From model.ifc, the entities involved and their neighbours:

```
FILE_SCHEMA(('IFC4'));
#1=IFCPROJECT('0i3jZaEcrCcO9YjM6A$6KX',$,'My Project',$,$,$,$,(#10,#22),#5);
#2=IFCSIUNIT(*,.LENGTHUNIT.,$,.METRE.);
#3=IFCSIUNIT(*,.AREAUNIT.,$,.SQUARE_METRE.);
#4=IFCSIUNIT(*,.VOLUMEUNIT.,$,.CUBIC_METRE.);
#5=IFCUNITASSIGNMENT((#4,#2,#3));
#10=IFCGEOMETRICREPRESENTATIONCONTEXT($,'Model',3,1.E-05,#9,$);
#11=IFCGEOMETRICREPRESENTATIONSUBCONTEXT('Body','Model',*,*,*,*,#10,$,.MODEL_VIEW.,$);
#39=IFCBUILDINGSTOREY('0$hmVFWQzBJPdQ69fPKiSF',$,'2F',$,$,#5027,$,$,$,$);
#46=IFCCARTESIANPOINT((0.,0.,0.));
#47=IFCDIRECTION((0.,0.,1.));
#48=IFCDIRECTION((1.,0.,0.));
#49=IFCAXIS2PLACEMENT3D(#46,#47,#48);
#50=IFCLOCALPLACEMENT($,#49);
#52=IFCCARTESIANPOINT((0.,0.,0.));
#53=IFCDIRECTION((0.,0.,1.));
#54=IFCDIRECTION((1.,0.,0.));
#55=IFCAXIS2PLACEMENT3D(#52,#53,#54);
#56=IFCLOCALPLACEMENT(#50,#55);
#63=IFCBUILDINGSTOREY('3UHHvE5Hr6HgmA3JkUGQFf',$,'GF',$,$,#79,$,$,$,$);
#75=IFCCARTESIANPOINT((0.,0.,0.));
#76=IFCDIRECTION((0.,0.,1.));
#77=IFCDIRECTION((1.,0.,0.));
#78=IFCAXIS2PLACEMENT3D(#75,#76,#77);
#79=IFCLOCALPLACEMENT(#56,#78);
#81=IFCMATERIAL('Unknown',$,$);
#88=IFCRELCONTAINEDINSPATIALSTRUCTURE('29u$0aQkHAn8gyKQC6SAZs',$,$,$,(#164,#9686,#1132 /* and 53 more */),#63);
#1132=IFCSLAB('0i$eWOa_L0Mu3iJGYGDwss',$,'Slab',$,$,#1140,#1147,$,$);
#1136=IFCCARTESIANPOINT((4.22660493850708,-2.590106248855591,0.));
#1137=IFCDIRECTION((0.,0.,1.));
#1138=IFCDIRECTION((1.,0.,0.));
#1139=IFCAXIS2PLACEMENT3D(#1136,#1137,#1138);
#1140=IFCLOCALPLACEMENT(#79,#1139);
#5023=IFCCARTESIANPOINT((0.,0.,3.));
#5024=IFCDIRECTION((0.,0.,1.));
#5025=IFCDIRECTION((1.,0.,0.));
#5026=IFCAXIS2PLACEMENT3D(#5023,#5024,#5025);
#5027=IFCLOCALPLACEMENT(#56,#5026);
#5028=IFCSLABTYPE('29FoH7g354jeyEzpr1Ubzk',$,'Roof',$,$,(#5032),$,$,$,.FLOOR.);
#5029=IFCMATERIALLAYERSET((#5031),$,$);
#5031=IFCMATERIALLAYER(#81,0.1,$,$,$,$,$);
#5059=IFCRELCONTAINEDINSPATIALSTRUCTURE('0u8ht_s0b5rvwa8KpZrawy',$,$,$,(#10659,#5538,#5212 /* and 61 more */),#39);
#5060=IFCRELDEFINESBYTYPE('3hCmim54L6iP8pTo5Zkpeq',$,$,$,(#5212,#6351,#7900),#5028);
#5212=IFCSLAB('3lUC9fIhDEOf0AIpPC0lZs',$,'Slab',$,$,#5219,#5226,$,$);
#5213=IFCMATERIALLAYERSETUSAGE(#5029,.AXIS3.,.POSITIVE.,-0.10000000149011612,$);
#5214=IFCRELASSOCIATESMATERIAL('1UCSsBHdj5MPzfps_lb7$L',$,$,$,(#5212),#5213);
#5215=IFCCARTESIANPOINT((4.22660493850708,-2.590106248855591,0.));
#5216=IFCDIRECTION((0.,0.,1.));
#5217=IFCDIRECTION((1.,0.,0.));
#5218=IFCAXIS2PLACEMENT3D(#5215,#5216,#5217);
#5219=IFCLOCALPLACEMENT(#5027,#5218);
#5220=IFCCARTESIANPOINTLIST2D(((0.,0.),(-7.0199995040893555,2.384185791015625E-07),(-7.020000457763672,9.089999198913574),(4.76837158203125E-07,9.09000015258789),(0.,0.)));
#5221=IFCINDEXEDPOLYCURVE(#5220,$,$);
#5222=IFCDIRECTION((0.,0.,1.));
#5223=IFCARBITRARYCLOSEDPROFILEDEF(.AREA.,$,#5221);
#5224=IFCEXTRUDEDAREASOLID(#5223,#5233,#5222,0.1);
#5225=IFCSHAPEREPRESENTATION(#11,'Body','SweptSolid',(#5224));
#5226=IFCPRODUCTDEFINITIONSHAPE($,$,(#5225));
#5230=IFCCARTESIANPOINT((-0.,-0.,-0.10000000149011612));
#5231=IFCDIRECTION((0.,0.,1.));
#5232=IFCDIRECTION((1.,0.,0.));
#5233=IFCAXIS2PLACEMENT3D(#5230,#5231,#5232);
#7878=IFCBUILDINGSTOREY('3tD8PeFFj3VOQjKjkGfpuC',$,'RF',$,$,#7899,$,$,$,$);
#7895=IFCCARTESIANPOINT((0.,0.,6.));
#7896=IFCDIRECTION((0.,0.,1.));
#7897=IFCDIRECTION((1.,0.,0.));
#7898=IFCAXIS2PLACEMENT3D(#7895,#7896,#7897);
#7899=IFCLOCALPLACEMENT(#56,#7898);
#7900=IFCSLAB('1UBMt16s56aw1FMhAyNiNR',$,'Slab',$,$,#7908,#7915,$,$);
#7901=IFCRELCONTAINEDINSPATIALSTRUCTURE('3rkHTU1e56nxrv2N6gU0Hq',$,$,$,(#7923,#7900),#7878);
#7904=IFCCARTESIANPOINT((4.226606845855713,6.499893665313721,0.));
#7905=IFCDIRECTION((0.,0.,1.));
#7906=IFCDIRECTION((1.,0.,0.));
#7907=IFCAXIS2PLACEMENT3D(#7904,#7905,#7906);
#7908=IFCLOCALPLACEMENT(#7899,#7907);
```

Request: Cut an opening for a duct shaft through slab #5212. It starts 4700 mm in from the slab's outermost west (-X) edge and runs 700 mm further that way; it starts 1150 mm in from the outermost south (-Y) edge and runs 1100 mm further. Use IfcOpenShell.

```python
import numpy as np
import ifcopenshell
import ifcopenshell.api.feature
import ifcopenshell.api.geometry
import ifcopenshell.api.root
import ifcopenshell.geom
import ifcopenshell.util.placement
import ifcopenshell.util.representation
import ifcopenshell.util.shape
import ifcopenshell.util.unit

model = ifcopenshell.open("model.ifc")
unit_scale = ifcopenshell.util.unit.calculate_unit_scale(model)
settings = ifcopenshell.geom.settings()


def volume(element):
    """Net volume in cubic metres, openings subtracted."""
    shape = ifcopenshell.geom.create_shape(settings, element)
    return ifcopenshell.util.shape.get_volume(shape.geometry)


slab = model.by_id(5212)
before = volume(slab)

# Extent in the slab's own axes, in metres. The edges named are its -X and -Y sides.
slab_shape = ifcopenshell.geom.create_shape(settings, slab)
vertices = ifcopenshell.util.shape.get_vertices(slab_shape.geometry)
x_min, y_min, bottom = vertices.min(axis=0)
top = vertices[:, 2].max()

opening = ifcopenshell.api.root.create_entity(model, ifc_class="IfcOpeningElement", name="Duct shaft opening", predefined_type="OPENING")
context = ifcopenshell.util.representation.get_context(model, "Model", "Body", "MODEL_VIEW")
width, depth = 0.7, 1.1
outline = [(0.0, 0.0), (width, 0.0), (width, depth), (0.0, depth), (0.0, 0.0)]
# Overshoot both faces by 50 mm so the cut is clean.
shape = ifcopenshell.api.geometry.add_slab_representation(
    model, context=context, depth=top - bottom + 0.1, polyline=outline
)
ifcopenshell.api.geometry.assign_representation(model, product=opening, representation=shape)

matrix = ifcopenshell.util.placement.get_local_placement(slab.ObjectPlacement)
matrix[:, 3] = matrix @ np.append(np.array([x_min + 4.7, y_min + 1.15, bottom - 0.05]) / unit_scale, 1.0)
ifcopenshell.api.geometry.edit_object_placement(model, product=opening, matrix=matrix, is_si=False)
ifcopenshell.api.feature.add_feature(model, feature=opening, element=slab)

after = volume(slab)

print(f"slab volume {before:.3f} -> {after:.3f} m3")

model.write("model_rev.ifc")
```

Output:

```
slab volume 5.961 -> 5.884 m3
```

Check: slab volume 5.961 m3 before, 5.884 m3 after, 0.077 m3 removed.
